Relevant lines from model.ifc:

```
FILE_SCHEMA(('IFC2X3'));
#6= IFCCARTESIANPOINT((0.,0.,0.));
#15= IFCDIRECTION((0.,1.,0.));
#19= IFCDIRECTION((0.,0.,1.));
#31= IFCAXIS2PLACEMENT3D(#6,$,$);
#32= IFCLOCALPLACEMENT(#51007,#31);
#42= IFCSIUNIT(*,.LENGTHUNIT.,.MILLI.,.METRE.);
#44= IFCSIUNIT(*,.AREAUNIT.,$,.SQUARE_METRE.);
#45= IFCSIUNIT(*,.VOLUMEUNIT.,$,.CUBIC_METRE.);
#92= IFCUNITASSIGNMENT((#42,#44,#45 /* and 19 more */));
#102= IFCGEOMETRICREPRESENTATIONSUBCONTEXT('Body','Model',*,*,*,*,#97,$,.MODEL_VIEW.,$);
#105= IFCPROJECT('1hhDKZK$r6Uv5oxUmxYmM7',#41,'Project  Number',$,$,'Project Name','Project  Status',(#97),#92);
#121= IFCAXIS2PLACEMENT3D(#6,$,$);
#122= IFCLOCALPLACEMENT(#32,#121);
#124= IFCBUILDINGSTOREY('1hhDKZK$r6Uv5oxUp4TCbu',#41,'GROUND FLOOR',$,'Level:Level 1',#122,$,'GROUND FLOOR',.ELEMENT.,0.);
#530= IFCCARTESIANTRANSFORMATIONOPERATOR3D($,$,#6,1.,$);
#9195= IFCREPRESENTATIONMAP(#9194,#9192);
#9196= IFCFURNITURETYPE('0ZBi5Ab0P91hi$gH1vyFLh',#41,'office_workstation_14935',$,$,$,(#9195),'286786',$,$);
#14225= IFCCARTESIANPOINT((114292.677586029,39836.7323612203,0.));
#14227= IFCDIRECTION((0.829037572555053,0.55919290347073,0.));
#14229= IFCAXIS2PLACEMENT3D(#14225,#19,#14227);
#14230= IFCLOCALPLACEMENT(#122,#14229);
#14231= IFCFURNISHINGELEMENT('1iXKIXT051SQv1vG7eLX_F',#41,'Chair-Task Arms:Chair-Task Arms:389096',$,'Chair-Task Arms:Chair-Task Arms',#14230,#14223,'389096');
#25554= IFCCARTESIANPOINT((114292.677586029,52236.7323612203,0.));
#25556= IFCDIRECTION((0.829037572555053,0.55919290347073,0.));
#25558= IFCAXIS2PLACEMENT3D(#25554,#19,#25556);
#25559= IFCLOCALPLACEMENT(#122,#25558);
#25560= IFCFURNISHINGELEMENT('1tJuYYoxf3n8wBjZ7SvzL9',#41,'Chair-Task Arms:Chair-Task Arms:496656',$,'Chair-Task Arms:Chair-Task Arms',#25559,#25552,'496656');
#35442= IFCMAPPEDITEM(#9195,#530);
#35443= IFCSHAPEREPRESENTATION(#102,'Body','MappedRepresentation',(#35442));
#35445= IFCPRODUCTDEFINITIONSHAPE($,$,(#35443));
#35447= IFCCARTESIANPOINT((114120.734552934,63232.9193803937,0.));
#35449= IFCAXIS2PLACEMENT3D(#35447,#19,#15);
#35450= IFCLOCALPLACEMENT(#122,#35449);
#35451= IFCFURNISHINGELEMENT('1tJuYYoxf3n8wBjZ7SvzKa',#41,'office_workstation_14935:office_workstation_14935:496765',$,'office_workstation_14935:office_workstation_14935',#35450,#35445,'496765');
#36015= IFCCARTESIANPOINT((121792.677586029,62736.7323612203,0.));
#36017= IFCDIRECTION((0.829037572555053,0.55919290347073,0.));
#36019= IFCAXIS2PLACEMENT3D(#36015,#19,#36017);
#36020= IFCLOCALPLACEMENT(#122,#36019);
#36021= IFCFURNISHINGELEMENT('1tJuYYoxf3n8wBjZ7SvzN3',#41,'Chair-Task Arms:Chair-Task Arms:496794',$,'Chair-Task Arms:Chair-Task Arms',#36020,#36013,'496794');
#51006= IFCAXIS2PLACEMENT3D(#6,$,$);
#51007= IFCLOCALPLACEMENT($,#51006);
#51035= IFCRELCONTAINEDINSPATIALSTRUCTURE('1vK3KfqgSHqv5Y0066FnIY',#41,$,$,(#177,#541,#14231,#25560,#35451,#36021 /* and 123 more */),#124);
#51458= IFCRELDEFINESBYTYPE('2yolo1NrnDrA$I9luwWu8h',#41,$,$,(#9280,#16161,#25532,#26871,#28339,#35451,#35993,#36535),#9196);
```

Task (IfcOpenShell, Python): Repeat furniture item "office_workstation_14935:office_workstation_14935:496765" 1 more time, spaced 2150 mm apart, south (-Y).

```python
import numpy as np
import ifcopenshell
import ifcopenshell.api.geometry
import ifcopenshell.api.root
import ifcopenshell.util.element
import ifcopenshell.util.placement

model = ifcopenshell.open("model.ifc")


def reuse_history(source, copy):
    """copy_class also copies each property set's owner history, people and application; keep the originals."""
    for rel in copy.IsDefinedBy:
        if rel.is_a("IfcRelDefinesByProperties") and (history := rel.RelatingPropertyDefinition.OwnerHistory):
            rel.RelatingPropertyDefinition.OwnerHistory = source.OwnerHistory
            ifcopenshell.util.element.remove_deep2(model, history)


source = model.by_guid("1tJuYYoxf3n8wBjZ7SvzKa")
base = ifcopenshell.util.placement.get_local_placement(source.ObjectPlacement)
step = np.array([0.0, -1.0, 0.0]) * 2150.0

for i in range(1, 2):
    copy = ifcopenshell.api.root.copy_class(model, product=source)
    copy.Representation = ifcopenshell.util.element.copy_deep(
        model, source.Representation, exclude=["IfcGeometricRepresentationContext", "IfcRepresentationMap"]
    )
    copy.Name = "office_workstation_14935:office_workstation_14935"
    copy.Tag = None
    reuse_history(source, copy)
    matrix = base.copy()
    matrix[:3, 3] += i * step
    print("added at", matrix[:3, 3].round(3) + 0.0)
    ifcopenshell.api.geometry.edit_object_placement(model, product=copy, matrix=matrix, is_si=False)

model.write("model_edited.ifc")
```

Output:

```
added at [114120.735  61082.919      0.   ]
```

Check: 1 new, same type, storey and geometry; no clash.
